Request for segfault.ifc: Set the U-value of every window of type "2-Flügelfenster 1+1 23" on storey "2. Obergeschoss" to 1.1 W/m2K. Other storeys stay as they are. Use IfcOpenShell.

First a look at what the model holds.

```python
import ifcopenshell
import ifcopenshell.util.element

model = ifcopenshell.open("segfault.ifc")
print(model.schema)
storey = next(s for s in model.by_type("IfcBuildingStorey") if s.Name == "2. Obergeschoss")
windows = [e for e in ifcopenshell.util.element.get_decomposition(storey) if e.is_a("IfcWindow")]
seen = {}
for e in windows:
    element_type = ifcopenshell.util.element.get_type(e)
    key = (element_type.Name if element_type != e and element_type else None, ifcopenshell.util.element.get_pset(e, "Pset_WindowCommon", "ThermalTransmittance"))
    seen[key] = seen.get(key, 0) + 1
for (name, value), count in sorted(seen.items(), key=str):
    print(count, "x", name, "|", value)
```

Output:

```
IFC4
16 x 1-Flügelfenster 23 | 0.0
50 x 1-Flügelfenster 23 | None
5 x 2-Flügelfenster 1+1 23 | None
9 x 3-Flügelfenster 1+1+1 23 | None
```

```python
import ifcopenshell
import ifcopenshell.api.pset
import ifcopenshell.util.element

model = ifcopenshell.open("segfault.ifc")

storey = next(s for s in model.by_type("IfcBuildingStorey") if s.Name == "2. Obergeschoss")
windows = [e for e in ifcopenshell.util.element.get_decomposition(storey) if e.is_a("IfcWindow")]

count = 0
for e in windows:
    element_type = ifcopenshell.util.element.get_type(e)
    if element_type in (None, e) or element_type.Name != "2-Flügelfenster 1+1 23":
        continue
    # add_pset returns the element's existing set when there is one.
    pset = ifcopenshell.api.pset.add_pset(model, product=e, name="Pset_WindowCommon")
    ifcopenshell.api.pset.edit_pset(model, pset=pset, properties={"ThermalTransmittance": 1.1})
    count += 1

print(count, "windows updated")

model.write("segfault_v2.ifc")
```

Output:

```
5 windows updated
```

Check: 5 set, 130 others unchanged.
